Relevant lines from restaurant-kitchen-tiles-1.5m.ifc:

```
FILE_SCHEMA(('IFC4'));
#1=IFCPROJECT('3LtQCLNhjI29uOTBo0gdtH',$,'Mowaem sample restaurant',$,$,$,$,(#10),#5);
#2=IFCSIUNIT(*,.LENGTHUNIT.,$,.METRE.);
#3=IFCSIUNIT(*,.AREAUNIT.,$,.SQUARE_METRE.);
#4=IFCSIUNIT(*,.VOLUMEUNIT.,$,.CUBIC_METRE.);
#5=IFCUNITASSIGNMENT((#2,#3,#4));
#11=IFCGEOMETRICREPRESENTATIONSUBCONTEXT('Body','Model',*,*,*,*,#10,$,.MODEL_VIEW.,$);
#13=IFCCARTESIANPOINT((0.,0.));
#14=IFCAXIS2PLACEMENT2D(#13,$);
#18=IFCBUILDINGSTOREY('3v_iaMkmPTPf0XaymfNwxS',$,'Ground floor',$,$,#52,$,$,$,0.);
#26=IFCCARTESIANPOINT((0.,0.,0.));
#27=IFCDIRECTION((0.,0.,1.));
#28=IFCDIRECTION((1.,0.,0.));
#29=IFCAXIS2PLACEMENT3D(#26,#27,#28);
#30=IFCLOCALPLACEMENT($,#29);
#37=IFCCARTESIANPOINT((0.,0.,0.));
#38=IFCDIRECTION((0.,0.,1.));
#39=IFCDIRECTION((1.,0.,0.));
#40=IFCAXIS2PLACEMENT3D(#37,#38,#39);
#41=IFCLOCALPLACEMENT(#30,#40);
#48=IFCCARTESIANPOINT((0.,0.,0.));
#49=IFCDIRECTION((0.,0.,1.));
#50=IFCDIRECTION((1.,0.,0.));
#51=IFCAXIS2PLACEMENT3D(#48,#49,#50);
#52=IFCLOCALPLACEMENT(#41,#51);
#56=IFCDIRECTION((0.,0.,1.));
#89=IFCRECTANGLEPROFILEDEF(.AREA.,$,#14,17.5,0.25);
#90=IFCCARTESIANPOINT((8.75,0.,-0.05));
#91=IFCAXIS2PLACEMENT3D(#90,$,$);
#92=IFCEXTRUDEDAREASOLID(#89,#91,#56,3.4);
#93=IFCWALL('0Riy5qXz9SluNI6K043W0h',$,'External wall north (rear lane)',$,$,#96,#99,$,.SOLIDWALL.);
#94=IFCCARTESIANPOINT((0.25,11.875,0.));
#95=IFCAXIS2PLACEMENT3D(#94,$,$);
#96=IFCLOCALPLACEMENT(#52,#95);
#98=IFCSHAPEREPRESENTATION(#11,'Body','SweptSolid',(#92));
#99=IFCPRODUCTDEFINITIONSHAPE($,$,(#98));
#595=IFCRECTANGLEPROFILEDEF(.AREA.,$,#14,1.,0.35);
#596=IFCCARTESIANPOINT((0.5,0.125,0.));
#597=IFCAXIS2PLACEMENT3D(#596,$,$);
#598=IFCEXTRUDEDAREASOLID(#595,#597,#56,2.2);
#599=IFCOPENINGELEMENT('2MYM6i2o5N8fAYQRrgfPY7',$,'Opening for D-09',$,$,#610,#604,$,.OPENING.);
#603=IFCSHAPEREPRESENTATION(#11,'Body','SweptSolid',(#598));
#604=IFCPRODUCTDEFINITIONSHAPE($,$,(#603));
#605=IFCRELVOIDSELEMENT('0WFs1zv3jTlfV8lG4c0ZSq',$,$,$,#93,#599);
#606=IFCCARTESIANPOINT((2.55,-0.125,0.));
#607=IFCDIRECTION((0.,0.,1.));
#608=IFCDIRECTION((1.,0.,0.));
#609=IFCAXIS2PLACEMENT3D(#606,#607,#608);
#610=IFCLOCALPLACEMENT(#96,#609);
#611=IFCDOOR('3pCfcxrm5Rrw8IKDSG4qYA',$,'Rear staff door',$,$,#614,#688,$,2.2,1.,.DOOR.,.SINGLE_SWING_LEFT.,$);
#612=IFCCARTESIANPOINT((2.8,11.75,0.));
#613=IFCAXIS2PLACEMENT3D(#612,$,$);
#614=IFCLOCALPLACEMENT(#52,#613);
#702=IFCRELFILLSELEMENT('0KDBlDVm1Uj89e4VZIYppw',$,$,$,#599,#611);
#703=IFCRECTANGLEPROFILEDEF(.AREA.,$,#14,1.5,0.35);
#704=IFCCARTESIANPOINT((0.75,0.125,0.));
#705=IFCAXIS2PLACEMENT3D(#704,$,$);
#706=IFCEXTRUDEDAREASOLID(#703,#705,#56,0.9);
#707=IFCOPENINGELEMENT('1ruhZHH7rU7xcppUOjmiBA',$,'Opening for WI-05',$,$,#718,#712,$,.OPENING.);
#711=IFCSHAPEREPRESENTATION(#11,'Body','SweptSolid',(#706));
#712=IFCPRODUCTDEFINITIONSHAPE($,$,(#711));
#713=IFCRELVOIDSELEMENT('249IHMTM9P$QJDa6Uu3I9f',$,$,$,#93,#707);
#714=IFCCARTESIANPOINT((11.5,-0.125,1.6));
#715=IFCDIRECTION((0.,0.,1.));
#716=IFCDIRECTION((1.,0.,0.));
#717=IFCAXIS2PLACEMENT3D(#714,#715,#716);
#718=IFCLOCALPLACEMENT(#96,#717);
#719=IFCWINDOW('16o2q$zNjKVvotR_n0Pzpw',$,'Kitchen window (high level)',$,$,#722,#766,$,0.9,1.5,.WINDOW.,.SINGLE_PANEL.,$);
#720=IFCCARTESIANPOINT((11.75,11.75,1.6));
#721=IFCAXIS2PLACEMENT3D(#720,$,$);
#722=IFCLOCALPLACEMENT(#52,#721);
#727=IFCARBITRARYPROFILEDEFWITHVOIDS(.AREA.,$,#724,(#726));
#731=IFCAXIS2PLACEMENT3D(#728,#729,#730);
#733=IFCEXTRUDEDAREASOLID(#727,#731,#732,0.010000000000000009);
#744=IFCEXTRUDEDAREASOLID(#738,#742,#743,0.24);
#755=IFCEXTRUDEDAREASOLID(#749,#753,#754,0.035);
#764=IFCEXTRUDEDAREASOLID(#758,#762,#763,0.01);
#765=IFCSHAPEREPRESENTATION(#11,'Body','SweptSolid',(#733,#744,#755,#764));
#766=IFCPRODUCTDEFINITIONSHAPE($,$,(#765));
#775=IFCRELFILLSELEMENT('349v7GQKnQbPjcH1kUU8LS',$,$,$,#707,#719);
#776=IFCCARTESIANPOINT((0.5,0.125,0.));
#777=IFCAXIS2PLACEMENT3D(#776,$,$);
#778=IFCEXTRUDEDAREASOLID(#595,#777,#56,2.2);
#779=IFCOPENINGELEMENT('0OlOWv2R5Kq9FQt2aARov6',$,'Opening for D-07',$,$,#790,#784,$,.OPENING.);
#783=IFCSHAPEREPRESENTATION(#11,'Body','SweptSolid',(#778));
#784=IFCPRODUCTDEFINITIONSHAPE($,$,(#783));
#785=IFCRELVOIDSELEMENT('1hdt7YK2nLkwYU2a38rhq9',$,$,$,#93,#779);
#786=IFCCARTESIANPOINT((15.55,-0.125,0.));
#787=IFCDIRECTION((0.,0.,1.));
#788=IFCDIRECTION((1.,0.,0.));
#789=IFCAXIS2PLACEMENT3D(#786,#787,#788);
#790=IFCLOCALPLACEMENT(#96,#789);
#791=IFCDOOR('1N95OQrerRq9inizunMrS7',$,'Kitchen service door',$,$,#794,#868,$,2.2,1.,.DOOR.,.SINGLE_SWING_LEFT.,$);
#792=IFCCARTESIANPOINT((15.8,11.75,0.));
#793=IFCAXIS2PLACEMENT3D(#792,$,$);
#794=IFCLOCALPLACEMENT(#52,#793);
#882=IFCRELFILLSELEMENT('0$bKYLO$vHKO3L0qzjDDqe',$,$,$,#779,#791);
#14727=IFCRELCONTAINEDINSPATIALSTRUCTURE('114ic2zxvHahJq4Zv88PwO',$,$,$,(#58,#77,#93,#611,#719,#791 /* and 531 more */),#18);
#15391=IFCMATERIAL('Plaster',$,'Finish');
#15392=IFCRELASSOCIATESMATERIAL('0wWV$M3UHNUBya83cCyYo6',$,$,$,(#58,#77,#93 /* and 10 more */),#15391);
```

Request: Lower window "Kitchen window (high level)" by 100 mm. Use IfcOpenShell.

```python
import numpy as np
import ifcopenshell
import ifcopenshell.api.geometry
import ifcopenshell.util.placement
import ifcopenshell.util.unit

model = ifcopenshell.open("restaurant-kitchen-tiles-1.5m.ifc")
unit_scale = ifcopenshell.util.unit.calculate_unit_scale(model)

window = model.by_guid("16o2q$zNjKVvotR_n0Pzpw")
opening = window.FillsVoids[0].RelatingOpeningElement
dz = -0.1

shift = np.array([0.0, 0.0, dz])
# The window is not placed relative to its opening, so move both.
for product in (opening, window):
    matrix = ifcopenshell.util.placement.get_local_placement(product.ObjectPlacement)
    matrix[:3, 3] += shift
    ifcopenshell.api.geometry.edit_object_placement(model, product=product, matrix=matrix, is_si=False)

print(f"moved by {dz * unit_scale:+.3f} m")

model.write("restaurant-kitchen-tiles-1.5m_rev.ifc")
```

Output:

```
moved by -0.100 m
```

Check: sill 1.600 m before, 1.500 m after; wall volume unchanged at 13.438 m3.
